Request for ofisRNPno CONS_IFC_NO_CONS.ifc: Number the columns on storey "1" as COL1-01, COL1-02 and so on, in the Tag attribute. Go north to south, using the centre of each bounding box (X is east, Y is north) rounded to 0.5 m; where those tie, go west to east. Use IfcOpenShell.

First a look at what the model holds.

```python
import ifcopenshell
import ifcopenshell.util.element
import ifcopenshell.util.placement

model = ifcopenshell.open("ofisRNPno CONS_IFC_NO_CONS.ifc")
print(model.schema)
storey = next(s for s in model.by_type("IfcBuildingStorey") if s.Name == "1")
columns = [e for e in ifcopenshell.util.element.get_decomposition(storey) if e.is_a("IfcColumn")]
for e in sorted(columns, key=lambda e: e.id()):
    origin = ifcopenshell.util.placement.get_local_placement(e.ObjectPlacement)[:3, 3]
    print(e.id(), e.Tag, e.Name, origin.round(2) + 0.0, sep=" | ")
```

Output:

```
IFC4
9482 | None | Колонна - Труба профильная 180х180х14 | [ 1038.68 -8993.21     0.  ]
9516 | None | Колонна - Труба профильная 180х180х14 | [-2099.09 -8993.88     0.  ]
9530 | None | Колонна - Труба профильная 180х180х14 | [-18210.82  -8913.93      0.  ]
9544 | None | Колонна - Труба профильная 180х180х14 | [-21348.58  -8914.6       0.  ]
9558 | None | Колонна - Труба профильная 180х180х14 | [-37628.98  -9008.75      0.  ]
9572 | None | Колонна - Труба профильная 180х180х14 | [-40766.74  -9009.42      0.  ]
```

```python
import ifcopenshell
import ifcopenshell.geom
import ifcopenshell.util.element
import ifcopenshell.util.shape

model = ifcopenshell.open("ofisRNPno CONS_IFC_NO_CONS.ifc")
settings = ifcopenshell.geom.settings()
settings.set("use-world-coords", True)


def centre(element):
    shape = ifcopenshell.geom.create_shape(settings, element)
    return ifcopenshell.util.shape.get_bbox_centroid(shape.geometry)


storey = next(s for s in model.by_type("IfcBuildingStorey") if s.Name == "1")
columns = [e for e in ifcopenshell.util.element.get_decomposition(storey) if e.is_a("IfcColumn")]

# Insertion points can sit at a corner or the storey origin, so sort by the geometry (in metres).
centres = {e: centre(e) for e in columns}
columns.sort(key=lambda e: (-round(centres[e][1] / 0.5), centres[e][0]))

for i, e in enumerate(columns, start=1):
    number = f"COL1-{i:02d}"
    e.Tag = number
    print(e.id(), number)

model.write("ofisRNPno CONS_IFC_NO_CONS-out.ifc")
```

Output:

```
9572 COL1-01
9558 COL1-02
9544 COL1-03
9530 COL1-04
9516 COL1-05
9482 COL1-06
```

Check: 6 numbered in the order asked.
